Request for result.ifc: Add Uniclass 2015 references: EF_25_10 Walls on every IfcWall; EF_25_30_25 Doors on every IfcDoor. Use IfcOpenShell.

First a look at what the model holds.

```python
import ifcopenshell

model = ifcopenshell.open("result.ifc")
print(model.schema)
print("classifications:", [c.Name for c in model.by_type("IfcClassification")])
for ifc_class in ("IfcDoor", "IfcRoof", "IfcStair", "IfcWall", "IfcWindow"):
    print(ifc_class, len(model.by_type(ifc_class)))
```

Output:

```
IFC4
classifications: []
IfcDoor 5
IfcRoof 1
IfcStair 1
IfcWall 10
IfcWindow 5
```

```python
import ifcopenshell
import ifcopenshell.api.classification

model = ifcopenshell.open("result.ifc")

system = ifcopenshell.api.classification.add_classification(model, classification="Uniclass 2015")

codes = {
    "IfcWall": ("EF_25_10", "Walls"),
    "IfcDoor": ("EF_25_30_25", "Doors"),
}
for ifc_class, (code, name) in codes.items():
    products = model.by_type(ifc_class)
    ifcopenshell.api.classification.add_reference(
        model, products=products, classification=system, identification=code, name=name
    )
    print(code, len(products))

model.write("result_rev.ifc")
```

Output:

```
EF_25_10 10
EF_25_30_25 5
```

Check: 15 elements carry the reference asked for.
